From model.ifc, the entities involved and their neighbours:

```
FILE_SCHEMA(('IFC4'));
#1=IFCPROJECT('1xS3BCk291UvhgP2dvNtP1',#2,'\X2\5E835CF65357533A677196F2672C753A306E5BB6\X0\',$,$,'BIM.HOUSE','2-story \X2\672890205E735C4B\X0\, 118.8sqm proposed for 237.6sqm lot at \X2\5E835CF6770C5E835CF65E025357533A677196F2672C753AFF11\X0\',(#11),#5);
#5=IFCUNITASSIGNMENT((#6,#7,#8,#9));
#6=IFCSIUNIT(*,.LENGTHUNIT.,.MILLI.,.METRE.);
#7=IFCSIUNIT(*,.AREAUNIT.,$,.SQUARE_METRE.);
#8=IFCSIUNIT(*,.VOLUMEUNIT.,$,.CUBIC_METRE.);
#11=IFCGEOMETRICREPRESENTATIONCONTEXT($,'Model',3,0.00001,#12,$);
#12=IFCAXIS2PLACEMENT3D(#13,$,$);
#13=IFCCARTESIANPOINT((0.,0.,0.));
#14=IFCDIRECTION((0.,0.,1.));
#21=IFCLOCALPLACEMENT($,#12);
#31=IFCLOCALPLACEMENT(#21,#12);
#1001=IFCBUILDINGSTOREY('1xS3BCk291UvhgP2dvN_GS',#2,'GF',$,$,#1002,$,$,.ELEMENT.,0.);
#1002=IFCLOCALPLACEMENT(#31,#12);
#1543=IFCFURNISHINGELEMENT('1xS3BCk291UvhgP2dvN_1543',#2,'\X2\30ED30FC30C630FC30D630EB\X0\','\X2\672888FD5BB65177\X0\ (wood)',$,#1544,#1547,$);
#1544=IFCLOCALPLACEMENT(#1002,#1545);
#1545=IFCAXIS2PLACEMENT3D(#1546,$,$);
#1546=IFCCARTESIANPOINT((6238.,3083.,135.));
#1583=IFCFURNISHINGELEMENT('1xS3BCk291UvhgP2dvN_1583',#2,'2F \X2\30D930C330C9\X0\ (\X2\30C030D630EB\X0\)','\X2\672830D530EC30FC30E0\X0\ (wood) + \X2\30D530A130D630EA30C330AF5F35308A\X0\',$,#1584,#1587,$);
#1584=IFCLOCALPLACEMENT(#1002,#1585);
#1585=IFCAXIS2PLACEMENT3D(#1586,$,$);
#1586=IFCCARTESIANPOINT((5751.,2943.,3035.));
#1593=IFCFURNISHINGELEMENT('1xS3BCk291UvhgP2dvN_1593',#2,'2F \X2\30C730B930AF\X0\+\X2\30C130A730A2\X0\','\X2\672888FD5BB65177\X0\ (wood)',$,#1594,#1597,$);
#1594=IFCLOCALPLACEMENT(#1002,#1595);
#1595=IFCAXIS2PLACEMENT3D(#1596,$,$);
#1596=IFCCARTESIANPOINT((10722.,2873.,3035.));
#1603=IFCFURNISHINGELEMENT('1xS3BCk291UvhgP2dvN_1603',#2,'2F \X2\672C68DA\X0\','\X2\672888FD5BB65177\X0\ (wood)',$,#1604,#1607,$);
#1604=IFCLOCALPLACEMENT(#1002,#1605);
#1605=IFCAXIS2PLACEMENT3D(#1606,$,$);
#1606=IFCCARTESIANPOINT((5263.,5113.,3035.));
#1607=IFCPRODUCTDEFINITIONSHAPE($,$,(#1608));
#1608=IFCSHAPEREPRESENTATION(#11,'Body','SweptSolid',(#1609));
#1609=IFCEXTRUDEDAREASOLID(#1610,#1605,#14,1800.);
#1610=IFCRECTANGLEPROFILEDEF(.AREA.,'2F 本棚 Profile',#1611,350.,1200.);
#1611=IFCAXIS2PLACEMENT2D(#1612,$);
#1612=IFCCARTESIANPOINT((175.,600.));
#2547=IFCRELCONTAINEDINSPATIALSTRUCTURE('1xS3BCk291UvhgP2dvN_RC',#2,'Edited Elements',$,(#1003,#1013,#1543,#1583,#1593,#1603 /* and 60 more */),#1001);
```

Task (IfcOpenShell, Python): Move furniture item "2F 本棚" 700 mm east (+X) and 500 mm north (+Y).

```python
import ifcopenshell
import ifcopenshell.api.geometry
import ifcopenshell.util.placement
import ifcopenshell.util.unit

model = ifcopenshell.open("model.ifc")
unit_scale = ifcopenshell.util.unit.calculate_unit_scale(model)

item = model.by_guid("1xS3BCk291UvhgP2dvN_1603")
matrix = ifcopenshell.util.placement.get_local_placement(item.ObjectPlacement)
matrix[0, 3] += 0.7 / unit_scale
matrix[1, 3] += 0.5 / unit_scale
ifcopenshell.api.geometry.edit_object_placement(model, product=item, matrix=matrix, is_si=False)

print(ifcopenshell.util.placement.get_local_placement(item.ObjectPlacement).round(3) + 0.0)

model.write("model_updated.ifc")
```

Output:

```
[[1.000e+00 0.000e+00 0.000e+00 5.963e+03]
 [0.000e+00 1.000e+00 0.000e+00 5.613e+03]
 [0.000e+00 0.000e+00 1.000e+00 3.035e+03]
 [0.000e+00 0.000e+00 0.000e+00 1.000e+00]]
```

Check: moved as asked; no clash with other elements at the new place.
